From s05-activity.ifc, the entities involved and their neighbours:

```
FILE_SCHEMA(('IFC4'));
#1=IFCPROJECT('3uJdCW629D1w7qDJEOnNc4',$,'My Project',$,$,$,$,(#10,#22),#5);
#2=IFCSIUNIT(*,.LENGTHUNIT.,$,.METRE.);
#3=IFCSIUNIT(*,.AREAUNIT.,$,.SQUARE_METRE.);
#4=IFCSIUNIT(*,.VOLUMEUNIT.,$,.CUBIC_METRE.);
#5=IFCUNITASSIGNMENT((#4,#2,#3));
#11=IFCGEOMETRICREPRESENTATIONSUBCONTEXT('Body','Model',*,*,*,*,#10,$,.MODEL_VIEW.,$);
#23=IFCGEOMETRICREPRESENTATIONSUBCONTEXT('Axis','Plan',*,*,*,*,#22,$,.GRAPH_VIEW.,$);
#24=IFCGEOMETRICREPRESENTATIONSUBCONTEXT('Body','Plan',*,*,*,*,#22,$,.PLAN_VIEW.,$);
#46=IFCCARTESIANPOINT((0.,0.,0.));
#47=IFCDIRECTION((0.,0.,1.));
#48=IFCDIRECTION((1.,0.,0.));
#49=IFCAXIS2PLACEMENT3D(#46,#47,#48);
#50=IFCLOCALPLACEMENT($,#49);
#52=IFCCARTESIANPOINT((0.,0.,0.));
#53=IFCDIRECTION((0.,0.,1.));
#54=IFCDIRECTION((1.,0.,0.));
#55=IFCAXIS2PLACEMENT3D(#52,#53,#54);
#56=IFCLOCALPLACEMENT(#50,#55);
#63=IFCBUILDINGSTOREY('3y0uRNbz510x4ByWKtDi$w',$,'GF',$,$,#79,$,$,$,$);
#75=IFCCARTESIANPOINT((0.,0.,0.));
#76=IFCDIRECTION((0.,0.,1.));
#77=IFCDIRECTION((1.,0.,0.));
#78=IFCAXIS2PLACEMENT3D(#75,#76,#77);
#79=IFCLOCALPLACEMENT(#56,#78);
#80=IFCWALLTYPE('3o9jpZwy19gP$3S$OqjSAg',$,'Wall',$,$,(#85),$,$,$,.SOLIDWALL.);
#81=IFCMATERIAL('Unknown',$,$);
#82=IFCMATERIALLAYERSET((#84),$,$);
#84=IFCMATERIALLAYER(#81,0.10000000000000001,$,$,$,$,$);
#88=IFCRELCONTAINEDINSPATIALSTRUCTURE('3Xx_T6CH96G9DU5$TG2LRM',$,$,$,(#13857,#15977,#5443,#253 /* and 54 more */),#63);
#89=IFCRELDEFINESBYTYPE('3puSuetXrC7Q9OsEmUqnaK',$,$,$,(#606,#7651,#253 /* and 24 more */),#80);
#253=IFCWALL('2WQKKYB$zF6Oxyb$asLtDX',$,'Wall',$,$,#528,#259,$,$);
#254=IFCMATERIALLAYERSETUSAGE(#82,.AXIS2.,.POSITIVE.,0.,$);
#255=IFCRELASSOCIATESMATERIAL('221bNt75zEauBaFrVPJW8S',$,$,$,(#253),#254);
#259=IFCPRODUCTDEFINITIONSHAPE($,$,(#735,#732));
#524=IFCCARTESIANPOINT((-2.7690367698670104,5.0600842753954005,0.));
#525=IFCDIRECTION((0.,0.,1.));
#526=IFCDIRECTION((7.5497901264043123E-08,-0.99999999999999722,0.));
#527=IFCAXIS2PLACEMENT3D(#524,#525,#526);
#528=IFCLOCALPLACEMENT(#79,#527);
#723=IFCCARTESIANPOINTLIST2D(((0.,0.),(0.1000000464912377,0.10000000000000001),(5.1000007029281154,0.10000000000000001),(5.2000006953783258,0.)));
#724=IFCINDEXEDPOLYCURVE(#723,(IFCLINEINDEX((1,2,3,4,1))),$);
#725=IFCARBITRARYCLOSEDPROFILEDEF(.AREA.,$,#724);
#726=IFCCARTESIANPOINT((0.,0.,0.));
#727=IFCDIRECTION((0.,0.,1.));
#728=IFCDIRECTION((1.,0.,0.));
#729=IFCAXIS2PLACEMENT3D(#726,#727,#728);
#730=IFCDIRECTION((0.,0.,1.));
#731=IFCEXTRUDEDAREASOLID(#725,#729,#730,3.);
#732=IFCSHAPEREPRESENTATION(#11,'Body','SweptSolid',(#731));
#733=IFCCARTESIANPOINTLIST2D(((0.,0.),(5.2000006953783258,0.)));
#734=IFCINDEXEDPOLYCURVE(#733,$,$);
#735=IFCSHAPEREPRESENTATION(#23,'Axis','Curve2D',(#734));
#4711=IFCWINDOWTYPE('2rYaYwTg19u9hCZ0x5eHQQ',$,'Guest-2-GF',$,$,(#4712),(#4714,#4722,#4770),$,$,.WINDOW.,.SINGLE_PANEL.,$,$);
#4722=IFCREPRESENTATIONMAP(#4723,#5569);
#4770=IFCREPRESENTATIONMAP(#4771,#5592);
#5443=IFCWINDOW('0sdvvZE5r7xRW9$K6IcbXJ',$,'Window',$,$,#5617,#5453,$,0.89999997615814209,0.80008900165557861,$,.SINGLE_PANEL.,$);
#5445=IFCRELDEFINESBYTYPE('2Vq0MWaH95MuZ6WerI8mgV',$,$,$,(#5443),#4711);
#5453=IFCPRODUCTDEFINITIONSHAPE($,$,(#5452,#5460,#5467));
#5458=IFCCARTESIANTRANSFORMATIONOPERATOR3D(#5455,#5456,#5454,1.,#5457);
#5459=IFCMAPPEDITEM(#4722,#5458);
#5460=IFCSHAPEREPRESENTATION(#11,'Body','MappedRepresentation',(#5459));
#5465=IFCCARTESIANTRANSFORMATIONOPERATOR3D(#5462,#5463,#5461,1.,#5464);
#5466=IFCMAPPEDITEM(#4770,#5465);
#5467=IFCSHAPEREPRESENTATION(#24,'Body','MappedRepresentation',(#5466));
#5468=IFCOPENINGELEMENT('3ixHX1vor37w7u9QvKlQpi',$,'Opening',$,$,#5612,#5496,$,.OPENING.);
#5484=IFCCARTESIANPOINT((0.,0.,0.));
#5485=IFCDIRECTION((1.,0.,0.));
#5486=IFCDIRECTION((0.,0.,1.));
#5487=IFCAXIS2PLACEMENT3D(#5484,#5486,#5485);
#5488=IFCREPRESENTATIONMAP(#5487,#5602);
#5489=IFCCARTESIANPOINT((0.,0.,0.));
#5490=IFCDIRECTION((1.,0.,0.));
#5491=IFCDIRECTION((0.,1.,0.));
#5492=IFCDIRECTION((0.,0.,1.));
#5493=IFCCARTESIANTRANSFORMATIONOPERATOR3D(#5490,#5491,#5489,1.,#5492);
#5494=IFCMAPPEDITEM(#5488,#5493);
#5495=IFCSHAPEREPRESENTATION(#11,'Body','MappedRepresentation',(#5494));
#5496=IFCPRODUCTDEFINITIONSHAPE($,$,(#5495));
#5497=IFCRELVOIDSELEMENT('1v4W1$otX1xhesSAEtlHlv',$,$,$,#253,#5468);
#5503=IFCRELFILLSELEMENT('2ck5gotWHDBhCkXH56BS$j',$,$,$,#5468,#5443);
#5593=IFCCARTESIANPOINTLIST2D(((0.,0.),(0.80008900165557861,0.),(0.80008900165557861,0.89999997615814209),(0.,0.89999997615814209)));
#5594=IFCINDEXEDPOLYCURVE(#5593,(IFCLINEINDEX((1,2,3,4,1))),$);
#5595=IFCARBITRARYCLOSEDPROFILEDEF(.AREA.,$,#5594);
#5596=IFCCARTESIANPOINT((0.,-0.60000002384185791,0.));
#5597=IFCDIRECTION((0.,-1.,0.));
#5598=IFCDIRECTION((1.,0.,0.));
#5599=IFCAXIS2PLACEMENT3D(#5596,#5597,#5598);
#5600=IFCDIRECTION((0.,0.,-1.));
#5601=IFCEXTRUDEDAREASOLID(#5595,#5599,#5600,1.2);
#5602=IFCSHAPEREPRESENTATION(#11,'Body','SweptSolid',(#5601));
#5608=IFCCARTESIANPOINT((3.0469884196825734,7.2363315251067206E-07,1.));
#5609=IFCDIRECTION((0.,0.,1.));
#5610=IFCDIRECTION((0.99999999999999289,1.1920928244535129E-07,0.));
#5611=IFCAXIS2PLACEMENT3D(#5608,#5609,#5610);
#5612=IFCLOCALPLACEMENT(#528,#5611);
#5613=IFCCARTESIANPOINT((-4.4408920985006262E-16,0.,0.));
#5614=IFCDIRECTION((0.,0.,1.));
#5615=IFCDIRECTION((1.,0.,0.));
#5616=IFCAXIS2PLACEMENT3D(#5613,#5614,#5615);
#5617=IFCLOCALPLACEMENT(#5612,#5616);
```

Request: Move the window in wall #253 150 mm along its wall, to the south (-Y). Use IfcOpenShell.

```python
import ifcopenshell
import ifcopenshell.api.geometry
import ifcopenshell.util.placement
import ifcopenshell.util.unit

model = ifcopenshell.open("s05-activity.ifc")
unit_scale = ifcopenshell.util.unit.calculate_unit_scale(model)

window = model.by_guid("0sdvvZE5r7xRW9$K6IcbXJ")
opening = window.FillsVoids[0].RelatingOpeningElement
wall = opening.VoidsElements[0].RelatingBuildingElement

wall_matrix = ifcopenshell.util.placement.get_local_placement(wall.ObjectPlacement)
shift = wall_matrix[:3, 0] * 0.15 / unit_scale
before = ifcopenshell.util.placement.get_local_placement(window.ObjectPlacement)[:3, 3].copy()

# The window is placed relative to its opening, so it follows when the opening moves.
matrix = ifcopenshell.util.placement.get_local_placement(opening.ObjectPlacement)
matrix[:3, 3] += shift
ifcopenshell.api.geometry.edit_object_placement(
    model, product=opening, matrix=matrix, is_si=False, should_transform_children=True
)

after = ifcopenshell.util.placement.get_local_placement(window.ObjectPlacement)[:3, 3]
print("window moved by", (after - before).round(3) + 0.0)

model.write("s05-activity-out.ifc")
```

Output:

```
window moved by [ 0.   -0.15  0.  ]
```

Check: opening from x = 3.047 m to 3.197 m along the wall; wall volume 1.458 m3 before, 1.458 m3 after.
